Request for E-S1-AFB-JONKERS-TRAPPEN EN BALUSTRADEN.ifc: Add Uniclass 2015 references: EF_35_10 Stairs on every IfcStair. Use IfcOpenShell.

First a look at what the model holds.

```python
import ifcopenshell

model = ifcopenshell.open("E-S1-AFB-JONKERS-TRAPPEN EN BALUSTRADEN.ifc")
print(model.schema)
print("classifications:", [c.Name for c in model.by_type("IfcClassification")])
for ifc_class in ("IfcDoor", "IfcRoof", "IfcStair", "IfcWall", "IfcWindow"):
    print(ifc_class, len(model.by_type(ifc_class)))
```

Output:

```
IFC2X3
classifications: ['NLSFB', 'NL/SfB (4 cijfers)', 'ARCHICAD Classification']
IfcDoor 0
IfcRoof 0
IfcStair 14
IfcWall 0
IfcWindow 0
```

```python
import ifcopenshell
import ifcopenshell.api.classification

model = ifcopenshell.open("E-S1-AFB-JONKERS-TRAPPEN EN BALUSTRADEN.ifc")

# IFC2X3 requires Source and Edition and has no link from the project to the system.
system = model.create_entity("IfcClassification", Source="NBS", Edition="2015", Name="Uniclass 2015")

codes = {
    "IfcStair": ("EF_35_10", "Stairs"),
}
for ifc_class, (code, name) in codes.items():
    products = model.by_type(ifc_class)
    ifcopenshell.api.classification.add_reference(
        model, products=products, classification=system, identification=code, name=name
    )
    print(code, len(products))

model.write("E-S1-AFB-JONKERS-TRAPPEN EN BALUSTRADEN_rev.ifc")
```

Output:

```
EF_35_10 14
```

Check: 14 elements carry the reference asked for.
